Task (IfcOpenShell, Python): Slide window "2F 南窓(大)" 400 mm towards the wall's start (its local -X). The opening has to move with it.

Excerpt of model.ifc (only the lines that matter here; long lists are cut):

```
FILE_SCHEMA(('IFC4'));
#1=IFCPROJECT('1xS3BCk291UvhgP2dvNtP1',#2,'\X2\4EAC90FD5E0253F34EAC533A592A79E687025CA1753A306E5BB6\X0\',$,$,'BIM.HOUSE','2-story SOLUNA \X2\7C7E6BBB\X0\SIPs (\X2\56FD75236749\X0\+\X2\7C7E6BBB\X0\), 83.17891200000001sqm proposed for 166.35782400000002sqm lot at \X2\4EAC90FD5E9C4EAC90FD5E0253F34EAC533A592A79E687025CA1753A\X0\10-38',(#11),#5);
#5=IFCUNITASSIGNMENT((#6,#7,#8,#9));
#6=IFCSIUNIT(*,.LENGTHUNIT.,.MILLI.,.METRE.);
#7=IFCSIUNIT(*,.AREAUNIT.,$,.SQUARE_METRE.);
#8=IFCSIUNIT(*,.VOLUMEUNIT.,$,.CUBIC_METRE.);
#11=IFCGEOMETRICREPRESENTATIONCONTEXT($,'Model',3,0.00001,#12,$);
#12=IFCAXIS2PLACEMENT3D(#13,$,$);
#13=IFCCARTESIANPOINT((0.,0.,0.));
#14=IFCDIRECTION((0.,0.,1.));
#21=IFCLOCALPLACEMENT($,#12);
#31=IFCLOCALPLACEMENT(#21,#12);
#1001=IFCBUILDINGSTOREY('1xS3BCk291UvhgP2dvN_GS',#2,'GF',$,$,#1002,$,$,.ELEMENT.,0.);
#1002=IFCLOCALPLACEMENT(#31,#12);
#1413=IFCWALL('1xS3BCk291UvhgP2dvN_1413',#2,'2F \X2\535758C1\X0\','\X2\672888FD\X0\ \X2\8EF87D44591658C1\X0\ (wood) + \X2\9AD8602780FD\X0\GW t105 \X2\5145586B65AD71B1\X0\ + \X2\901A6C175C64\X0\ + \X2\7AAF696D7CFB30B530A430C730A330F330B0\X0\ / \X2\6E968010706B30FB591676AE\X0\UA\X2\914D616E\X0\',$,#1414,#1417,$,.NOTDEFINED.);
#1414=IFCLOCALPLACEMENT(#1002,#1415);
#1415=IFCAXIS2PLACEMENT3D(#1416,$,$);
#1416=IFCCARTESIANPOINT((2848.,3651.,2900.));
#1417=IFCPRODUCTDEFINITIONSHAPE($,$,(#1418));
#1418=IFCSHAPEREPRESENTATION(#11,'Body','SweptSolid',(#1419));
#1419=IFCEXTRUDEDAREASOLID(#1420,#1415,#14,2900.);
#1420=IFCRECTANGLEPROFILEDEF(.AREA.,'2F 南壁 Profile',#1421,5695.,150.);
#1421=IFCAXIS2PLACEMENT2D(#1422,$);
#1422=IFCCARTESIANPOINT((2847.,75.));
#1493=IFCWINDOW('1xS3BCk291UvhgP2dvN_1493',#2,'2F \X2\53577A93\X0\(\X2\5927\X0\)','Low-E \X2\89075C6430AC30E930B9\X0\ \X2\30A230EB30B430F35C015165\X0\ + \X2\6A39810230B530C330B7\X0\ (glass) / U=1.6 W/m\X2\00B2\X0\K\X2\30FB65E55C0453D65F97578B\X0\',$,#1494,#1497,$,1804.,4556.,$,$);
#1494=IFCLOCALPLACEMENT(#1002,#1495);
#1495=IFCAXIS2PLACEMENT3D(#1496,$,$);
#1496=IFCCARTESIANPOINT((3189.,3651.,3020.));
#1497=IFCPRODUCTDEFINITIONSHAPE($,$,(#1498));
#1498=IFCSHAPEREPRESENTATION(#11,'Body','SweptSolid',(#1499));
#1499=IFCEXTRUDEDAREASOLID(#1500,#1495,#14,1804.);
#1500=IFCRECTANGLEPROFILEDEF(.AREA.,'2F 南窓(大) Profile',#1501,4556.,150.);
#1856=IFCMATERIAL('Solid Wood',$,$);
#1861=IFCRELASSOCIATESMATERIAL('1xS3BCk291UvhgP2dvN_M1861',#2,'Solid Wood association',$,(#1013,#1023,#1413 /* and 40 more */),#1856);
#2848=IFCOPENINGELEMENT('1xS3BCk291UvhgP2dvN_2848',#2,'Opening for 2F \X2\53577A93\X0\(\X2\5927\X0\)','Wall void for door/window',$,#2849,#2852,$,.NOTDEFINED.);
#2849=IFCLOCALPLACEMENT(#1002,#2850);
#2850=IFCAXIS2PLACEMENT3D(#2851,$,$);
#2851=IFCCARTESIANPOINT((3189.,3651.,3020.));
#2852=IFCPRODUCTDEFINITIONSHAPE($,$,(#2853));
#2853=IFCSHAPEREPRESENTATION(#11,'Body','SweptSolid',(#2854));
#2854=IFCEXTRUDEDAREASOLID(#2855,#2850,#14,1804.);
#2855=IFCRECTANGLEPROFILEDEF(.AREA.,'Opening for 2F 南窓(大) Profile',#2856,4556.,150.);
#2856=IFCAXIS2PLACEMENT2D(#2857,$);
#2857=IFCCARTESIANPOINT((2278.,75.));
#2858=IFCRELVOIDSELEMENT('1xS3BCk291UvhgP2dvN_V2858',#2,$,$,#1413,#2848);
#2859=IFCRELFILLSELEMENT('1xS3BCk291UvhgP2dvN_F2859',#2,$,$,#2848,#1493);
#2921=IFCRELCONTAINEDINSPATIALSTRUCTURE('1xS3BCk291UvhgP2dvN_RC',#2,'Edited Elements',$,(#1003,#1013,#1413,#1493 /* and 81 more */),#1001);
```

```python
import ifcopenshell
import ifcopenshell.api.geometry
import ifcopenshell.util.placement
import ifcopenshell.util.unit

model = ifcopenshell.open("model.ifc")
unit_scale = ifcopenshell.util.unit.calculate_unit_scale(model)

window = model.by_guid("1xS3BCk291UvhgP2dvN_1493")
opening = window.FillsVoids[0].RelatingOpeningElement
wall = opening.VoidsElements[0].RelatingBuildingElement

wall_matrix = ifcopenshell.util.placement.get_local_placement(wall.ObjectPlacement)
shift = wall_matrix[:3, 0] * -0.4 / unit_scale
before = ifcopenshell.util.placement.get_local_placement(window.ObjectPlacement)[:3, 3].copy()

# The window is not placed relative to its opening, so move both.
for product in (opening, window):
    matrix = ifcopenshell.util.placement.get_local_placement(product.ObjectPlacement)
    matrix[:3, 3] += shift
    ifcopenshell.api.geometry.edit_object_placement(model, product=product, matrix=matrix, is_si=False)

after = ifcopenshell.util.placement.get_local_placement(window.ObjectPlacement)[:3, 3]
print("window moved by", (after - before).round(3) + 0.0)

model.write("model_updated.ifc")
```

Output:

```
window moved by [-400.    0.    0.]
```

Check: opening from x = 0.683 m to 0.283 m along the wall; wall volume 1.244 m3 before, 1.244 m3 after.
